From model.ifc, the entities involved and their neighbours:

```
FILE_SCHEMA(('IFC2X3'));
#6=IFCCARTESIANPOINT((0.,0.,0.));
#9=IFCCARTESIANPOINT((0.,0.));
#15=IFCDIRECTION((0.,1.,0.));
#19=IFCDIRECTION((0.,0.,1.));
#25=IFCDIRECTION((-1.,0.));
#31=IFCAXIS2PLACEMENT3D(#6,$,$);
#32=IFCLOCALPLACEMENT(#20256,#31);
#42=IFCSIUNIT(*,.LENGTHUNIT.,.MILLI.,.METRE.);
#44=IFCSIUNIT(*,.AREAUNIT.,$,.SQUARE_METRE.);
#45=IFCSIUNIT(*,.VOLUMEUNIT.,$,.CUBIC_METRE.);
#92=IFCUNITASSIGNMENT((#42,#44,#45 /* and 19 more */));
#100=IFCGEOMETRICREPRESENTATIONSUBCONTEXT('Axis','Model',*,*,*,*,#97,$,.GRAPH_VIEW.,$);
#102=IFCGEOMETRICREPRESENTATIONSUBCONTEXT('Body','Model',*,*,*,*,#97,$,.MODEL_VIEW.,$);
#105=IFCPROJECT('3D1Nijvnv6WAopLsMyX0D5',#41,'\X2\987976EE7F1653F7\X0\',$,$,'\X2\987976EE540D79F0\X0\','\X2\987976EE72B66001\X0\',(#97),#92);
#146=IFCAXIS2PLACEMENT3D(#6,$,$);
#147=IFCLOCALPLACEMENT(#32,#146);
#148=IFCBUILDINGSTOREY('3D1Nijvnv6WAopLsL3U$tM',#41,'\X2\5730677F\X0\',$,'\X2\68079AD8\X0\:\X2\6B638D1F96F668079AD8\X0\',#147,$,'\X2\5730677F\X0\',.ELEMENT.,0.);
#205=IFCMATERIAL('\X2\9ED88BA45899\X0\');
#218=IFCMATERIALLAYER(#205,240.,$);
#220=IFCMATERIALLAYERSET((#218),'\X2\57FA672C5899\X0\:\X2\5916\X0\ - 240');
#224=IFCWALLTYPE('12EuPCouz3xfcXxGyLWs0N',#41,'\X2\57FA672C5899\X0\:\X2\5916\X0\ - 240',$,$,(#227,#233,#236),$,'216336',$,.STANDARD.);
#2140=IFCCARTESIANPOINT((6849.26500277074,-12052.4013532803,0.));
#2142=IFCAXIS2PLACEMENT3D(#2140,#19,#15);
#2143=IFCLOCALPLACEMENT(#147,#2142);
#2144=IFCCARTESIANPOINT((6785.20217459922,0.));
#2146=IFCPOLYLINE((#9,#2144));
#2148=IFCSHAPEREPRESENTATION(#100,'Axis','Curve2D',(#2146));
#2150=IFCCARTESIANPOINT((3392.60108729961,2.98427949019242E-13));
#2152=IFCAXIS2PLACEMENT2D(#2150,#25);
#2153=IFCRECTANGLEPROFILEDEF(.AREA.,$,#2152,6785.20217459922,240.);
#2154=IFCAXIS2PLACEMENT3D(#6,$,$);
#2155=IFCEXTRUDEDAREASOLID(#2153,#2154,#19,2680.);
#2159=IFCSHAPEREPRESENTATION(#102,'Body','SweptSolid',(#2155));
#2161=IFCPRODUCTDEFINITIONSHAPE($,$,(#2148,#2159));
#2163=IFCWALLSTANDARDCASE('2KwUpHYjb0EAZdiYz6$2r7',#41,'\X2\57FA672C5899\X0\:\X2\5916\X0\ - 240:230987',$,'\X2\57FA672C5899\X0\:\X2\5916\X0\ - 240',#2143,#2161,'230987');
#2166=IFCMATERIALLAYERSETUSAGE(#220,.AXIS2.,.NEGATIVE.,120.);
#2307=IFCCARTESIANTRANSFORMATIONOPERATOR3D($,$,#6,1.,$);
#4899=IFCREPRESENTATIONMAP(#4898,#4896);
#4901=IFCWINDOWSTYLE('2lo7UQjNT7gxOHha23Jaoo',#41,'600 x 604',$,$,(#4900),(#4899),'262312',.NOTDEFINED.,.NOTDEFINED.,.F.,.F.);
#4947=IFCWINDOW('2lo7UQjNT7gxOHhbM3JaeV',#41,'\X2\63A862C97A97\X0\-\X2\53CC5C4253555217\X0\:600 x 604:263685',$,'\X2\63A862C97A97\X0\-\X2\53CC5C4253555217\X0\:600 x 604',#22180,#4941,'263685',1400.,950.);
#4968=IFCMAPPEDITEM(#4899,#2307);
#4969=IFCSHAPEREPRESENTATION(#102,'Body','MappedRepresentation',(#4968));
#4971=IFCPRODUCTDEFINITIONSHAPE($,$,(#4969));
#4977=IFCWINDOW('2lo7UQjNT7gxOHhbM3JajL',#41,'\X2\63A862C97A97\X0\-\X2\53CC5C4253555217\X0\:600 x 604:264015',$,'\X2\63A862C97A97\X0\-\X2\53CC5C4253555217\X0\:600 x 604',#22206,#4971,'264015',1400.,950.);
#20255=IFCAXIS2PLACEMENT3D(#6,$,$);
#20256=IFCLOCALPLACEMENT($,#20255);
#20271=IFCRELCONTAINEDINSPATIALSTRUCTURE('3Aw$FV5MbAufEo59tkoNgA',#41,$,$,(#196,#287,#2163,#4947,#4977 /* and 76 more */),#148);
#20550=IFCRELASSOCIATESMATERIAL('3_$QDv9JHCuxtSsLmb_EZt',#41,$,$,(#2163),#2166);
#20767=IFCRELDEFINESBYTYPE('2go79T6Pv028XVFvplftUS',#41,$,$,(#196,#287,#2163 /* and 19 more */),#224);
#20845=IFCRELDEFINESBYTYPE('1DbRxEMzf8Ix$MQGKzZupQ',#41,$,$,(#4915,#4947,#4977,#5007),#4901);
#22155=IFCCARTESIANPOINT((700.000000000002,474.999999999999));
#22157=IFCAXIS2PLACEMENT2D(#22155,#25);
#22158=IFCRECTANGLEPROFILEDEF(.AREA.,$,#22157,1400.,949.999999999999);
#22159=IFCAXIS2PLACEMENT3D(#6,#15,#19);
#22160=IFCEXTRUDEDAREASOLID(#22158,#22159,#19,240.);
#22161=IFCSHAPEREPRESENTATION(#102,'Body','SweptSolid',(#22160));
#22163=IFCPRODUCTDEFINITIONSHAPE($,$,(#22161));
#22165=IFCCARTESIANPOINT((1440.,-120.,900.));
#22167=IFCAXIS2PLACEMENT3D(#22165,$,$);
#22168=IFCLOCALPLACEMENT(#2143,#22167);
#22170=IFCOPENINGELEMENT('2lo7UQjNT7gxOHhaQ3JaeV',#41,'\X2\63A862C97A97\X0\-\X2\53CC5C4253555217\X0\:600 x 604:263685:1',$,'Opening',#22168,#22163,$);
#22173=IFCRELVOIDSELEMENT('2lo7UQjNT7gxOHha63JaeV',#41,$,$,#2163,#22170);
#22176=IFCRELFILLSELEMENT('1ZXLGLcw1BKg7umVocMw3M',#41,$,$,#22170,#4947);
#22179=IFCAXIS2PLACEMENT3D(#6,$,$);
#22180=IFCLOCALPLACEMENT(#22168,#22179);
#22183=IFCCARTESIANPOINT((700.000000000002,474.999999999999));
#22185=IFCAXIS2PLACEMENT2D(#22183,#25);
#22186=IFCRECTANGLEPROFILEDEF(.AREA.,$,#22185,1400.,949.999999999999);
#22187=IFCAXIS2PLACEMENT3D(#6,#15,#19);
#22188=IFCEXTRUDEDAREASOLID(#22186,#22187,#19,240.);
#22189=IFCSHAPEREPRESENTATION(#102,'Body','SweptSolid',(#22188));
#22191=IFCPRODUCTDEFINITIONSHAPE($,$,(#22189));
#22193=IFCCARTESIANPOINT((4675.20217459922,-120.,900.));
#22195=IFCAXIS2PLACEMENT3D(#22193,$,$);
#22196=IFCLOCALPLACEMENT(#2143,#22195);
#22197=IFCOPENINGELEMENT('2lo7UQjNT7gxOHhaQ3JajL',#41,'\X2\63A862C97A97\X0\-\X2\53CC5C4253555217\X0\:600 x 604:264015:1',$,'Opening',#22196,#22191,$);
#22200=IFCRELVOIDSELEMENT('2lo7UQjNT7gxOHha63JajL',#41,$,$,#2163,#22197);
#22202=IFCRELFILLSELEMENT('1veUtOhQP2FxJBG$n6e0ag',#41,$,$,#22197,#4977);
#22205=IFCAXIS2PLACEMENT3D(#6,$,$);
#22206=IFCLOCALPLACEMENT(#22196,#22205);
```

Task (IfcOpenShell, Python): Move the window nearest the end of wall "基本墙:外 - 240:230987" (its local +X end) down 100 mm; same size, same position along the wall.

```python
import numpy as np
import ifcopenshell
import ifcopenshell.api.geometry
import ifcopenshell.util.placement
import ifcopenshell.util.unit

model = ifcopenshell.open("model.ifc")
unit_scale = ifcopenshell.util.unit.calculate_unit_scale(model)

window = model.by_id(4977)
opening = window.FillsVoids[0].RelatingOpeningElement
dz = -0.1 / unit_scale

shift = np.array([0.0, 0.0, dz])
# The window is placed relative to its opening, so it follows when the opening moves.
matrix = ifcopenshell.util.placement.get_local_placement(opening.ObjectPlacement)
matrix[:3, 3] += shift
ifcopenshell.api.geometry.edit_object_placement(
    model, product=opening, matrix=matrix, is_si=False, should_transform_children=True
)

print(f"moved by {dz * unit_scale:+.3f} m")

model.write("model-out.ifc")
```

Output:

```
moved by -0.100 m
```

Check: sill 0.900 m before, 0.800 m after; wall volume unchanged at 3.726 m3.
